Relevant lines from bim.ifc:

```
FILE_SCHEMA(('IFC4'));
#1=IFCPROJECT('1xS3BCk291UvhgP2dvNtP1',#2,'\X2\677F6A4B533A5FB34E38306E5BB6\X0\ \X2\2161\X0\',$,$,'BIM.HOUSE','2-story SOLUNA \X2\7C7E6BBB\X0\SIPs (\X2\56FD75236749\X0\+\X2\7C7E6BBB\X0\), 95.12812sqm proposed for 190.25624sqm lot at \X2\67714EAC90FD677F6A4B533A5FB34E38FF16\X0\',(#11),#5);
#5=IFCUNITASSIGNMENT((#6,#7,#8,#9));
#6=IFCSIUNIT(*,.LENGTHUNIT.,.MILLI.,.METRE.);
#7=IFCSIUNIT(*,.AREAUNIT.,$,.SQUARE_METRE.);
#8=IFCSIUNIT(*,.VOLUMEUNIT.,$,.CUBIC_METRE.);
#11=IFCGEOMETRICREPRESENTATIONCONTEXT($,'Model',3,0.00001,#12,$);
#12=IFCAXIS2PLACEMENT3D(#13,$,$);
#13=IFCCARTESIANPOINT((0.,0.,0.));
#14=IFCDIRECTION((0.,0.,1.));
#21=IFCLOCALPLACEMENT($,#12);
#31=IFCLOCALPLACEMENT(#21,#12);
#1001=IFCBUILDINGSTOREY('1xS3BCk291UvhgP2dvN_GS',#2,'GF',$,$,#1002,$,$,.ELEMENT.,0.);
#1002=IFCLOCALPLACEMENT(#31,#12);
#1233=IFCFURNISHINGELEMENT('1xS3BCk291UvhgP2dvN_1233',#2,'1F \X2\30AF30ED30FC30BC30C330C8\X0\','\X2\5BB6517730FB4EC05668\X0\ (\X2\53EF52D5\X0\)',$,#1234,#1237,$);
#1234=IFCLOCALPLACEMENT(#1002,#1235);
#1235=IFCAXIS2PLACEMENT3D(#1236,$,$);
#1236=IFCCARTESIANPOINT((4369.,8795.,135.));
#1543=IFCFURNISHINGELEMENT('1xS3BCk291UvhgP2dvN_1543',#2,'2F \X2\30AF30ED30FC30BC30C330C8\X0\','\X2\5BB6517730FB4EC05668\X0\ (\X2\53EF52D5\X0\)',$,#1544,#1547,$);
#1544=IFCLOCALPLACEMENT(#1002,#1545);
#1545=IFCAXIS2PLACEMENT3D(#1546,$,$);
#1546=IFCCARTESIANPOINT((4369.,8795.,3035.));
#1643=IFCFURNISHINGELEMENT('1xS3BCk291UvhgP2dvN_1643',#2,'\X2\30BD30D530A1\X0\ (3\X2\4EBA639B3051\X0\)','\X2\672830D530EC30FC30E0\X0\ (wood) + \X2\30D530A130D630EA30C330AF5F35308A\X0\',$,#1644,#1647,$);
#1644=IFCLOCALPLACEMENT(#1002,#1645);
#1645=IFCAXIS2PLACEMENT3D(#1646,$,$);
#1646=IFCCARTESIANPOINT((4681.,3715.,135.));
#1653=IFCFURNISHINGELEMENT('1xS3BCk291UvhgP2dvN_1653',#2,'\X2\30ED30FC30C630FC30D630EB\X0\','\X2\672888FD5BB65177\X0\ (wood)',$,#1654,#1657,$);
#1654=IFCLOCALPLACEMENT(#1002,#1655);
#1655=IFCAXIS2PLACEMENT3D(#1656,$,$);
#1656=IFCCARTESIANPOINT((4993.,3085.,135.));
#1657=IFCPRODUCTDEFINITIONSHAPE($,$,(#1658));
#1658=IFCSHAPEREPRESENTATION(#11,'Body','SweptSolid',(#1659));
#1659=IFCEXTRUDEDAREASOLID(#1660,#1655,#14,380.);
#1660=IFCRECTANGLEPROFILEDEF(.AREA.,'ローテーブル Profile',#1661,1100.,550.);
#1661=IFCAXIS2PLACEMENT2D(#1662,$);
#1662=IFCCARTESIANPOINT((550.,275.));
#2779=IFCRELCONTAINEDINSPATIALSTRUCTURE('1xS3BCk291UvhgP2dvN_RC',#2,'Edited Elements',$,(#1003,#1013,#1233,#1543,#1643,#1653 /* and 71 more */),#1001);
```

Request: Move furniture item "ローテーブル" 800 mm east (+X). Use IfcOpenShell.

```python
import ifcopenshell
import ifcopenshell.api.geometry
import ifcopenshell.util.placement
import ifcopenshell.util.unit

model = ifcopenshell.open("bim.ifc")
unit_scale = ifcopenshell.util.unit.calculate_unit_scale(model)

item = model.by_guid("1xS3BCk291UvhgP2dvN_1653")
matrix = ifcopenshell.util.placement.get_local_placement(item.ObjectPlacement)
matrix[0, 3] += 0.8 / unit_scale
ifcopenshell.api.geometry.edit_object_placement(model, product=item, matrix=matrix, is_si=False)

print(ifcopenshell.util.placement.get_local_placement(item.ObjectPlacement).round(3) + 0.0)

model.write("bim-out.ifc")
```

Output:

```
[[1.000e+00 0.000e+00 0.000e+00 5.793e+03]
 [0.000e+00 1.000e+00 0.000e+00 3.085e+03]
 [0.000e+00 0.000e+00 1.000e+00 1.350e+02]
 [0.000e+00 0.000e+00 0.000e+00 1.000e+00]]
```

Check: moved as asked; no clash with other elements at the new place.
